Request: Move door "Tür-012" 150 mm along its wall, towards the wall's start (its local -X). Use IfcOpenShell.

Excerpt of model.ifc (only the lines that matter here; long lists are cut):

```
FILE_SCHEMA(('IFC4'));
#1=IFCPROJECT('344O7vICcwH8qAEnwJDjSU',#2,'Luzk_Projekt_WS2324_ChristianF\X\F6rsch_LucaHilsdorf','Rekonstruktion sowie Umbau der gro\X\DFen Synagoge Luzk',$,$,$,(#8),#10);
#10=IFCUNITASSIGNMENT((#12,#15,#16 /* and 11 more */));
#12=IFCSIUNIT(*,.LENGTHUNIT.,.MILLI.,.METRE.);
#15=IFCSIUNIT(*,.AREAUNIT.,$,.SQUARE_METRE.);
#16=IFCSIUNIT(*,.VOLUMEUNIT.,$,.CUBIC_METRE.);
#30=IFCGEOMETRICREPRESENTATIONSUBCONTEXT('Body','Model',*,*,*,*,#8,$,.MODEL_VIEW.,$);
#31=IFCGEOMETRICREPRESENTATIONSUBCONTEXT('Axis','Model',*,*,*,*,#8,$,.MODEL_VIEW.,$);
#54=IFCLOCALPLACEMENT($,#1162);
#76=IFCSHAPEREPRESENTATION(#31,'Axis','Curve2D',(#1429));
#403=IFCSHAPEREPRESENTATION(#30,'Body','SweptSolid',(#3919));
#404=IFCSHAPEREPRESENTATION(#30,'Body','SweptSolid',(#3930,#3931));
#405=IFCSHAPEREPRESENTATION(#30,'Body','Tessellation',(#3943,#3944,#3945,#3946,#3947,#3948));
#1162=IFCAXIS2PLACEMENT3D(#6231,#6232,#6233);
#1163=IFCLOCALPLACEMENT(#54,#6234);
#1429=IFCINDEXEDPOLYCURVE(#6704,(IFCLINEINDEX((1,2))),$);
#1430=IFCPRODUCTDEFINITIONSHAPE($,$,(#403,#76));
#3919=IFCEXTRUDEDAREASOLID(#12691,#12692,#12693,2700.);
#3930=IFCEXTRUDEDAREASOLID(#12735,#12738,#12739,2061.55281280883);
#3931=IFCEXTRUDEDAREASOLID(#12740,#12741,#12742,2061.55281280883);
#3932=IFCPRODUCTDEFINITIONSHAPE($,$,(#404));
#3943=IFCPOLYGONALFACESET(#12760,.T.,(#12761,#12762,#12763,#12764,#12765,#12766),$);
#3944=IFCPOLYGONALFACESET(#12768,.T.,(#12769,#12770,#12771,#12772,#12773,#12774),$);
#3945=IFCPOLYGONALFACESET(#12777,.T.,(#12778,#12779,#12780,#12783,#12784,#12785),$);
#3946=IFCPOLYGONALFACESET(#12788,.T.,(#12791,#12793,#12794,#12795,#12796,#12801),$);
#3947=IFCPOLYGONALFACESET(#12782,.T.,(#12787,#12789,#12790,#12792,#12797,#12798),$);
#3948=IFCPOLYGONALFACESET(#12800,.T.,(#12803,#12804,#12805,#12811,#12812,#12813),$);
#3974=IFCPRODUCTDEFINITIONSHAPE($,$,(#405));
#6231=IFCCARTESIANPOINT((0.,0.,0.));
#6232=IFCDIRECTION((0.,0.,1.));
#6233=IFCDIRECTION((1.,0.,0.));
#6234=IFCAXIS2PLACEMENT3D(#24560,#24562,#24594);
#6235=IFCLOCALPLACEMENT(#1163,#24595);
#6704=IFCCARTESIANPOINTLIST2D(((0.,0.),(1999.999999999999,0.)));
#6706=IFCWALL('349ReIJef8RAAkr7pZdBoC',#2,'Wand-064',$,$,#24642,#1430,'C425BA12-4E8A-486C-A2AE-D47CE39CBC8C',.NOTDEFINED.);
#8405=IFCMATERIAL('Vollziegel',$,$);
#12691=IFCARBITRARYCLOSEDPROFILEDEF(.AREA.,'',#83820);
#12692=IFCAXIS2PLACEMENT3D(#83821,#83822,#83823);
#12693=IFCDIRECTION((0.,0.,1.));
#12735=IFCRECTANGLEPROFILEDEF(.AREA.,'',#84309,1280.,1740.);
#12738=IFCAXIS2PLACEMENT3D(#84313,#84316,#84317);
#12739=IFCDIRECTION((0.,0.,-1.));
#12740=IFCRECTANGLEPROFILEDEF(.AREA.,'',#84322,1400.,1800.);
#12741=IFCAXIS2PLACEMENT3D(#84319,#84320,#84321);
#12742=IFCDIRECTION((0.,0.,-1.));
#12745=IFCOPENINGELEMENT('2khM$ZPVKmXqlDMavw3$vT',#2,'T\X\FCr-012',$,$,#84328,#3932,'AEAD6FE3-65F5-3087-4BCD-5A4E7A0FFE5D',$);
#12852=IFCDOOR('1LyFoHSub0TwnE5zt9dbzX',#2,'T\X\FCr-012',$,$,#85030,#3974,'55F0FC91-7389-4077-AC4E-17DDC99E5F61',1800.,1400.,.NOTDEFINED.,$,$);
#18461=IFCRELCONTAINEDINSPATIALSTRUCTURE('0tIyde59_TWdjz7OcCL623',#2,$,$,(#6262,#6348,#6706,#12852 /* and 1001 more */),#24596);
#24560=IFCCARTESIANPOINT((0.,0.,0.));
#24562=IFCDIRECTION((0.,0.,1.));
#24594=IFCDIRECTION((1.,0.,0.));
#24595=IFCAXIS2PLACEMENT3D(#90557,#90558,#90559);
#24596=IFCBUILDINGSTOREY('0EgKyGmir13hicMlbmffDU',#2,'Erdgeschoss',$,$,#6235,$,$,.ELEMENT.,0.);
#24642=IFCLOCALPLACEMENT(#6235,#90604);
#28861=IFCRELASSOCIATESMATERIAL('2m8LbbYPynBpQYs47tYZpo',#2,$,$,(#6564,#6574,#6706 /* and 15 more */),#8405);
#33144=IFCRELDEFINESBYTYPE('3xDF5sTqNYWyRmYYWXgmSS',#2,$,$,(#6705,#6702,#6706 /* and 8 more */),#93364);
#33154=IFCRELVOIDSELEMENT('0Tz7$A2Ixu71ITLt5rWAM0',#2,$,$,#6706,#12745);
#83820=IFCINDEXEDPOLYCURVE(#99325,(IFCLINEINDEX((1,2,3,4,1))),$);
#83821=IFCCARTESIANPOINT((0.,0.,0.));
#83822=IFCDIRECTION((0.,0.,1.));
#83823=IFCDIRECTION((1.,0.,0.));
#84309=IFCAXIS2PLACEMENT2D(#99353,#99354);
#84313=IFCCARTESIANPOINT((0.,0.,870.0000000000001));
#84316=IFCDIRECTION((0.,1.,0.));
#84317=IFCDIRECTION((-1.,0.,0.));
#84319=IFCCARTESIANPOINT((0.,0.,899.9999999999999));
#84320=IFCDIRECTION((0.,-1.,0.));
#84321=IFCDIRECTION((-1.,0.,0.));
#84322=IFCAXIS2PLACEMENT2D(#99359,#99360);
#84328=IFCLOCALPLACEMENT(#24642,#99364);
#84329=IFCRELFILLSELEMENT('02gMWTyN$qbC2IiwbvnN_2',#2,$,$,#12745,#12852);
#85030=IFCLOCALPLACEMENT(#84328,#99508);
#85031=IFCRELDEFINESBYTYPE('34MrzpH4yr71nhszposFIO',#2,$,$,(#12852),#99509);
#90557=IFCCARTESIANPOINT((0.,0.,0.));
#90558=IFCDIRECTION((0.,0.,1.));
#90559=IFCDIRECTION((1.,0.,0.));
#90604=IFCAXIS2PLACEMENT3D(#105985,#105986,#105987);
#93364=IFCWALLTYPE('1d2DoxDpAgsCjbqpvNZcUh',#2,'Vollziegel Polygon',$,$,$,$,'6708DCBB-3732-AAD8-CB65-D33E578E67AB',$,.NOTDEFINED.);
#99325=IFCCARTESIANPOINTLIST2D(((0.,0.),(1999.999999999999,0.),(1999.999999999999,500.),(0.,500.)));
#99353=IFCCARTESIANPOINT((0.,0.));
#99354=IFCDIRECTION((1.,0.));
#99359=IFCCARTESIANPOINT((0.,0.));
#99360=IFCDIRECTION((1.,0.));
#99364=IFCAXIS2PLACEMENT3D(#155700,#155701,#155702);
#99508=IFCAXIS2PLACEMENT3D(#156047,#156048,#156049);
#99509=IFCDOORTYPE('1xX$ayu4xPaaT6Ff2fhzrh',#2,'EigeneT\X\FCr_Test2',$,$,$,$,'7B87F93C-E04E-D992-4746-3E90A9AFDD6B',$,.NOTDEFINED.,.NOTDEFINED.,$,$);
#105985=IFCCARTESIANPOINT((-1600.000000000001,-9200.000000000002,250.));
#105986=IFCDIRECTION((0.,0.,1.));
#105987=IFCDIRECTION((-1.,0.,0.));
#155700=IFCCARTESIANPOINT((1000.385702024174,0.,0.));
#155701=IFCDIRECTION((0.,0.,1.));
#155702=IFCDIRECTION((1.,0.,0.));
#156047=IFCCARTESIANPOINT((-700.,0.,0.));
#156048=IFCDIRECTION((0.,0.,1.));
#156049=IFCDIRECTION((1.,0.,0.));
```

```python
import ifcopenshell
import ifcopenshell.api.geometry
import ifcopenshell.util.placement

model = ifcopenshell.open("model.ifc")

door = model.by_guid("1LyFoHSub0TwnE5zt9dbzX")
opening = door.FillsVoids[0].RelatingOpeningElement
wall = opening.VoidsElements[0].RelatingBuildingElement

wall_matrix = ifcopenshell.util.placement.get_local_placement(wall.ObjectPlacement)
shift = wall_matrix[:3, 0] * -150.0
before = ifcopenshell.util.placement.get_local_placement(door.ObjectPlacement)[:3, 3].copy()

# The door is placed relative to its opening, so it follows when the opening moves.
matrix = ifcopenshell.util.placement.get_local_placement(opening.ObjectPlacement)
matrix[:3, 3] += shift
ifcopenshell.api.geometry.edit_object_placement(
    model, product=opening, matrix=matrix, is_si=False, should_transform_children=True
)

after = ifcopenshell.util.placement.get_local_placement(door.ObjectPlacement)[:3, 3]
print("door moved by", (after - before).round(3) + 0.0)

model.write("model-out.ifc")
```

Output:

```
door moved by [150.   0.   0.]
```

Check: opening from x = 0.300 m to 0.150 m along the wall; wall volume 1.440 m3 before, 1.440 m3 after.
